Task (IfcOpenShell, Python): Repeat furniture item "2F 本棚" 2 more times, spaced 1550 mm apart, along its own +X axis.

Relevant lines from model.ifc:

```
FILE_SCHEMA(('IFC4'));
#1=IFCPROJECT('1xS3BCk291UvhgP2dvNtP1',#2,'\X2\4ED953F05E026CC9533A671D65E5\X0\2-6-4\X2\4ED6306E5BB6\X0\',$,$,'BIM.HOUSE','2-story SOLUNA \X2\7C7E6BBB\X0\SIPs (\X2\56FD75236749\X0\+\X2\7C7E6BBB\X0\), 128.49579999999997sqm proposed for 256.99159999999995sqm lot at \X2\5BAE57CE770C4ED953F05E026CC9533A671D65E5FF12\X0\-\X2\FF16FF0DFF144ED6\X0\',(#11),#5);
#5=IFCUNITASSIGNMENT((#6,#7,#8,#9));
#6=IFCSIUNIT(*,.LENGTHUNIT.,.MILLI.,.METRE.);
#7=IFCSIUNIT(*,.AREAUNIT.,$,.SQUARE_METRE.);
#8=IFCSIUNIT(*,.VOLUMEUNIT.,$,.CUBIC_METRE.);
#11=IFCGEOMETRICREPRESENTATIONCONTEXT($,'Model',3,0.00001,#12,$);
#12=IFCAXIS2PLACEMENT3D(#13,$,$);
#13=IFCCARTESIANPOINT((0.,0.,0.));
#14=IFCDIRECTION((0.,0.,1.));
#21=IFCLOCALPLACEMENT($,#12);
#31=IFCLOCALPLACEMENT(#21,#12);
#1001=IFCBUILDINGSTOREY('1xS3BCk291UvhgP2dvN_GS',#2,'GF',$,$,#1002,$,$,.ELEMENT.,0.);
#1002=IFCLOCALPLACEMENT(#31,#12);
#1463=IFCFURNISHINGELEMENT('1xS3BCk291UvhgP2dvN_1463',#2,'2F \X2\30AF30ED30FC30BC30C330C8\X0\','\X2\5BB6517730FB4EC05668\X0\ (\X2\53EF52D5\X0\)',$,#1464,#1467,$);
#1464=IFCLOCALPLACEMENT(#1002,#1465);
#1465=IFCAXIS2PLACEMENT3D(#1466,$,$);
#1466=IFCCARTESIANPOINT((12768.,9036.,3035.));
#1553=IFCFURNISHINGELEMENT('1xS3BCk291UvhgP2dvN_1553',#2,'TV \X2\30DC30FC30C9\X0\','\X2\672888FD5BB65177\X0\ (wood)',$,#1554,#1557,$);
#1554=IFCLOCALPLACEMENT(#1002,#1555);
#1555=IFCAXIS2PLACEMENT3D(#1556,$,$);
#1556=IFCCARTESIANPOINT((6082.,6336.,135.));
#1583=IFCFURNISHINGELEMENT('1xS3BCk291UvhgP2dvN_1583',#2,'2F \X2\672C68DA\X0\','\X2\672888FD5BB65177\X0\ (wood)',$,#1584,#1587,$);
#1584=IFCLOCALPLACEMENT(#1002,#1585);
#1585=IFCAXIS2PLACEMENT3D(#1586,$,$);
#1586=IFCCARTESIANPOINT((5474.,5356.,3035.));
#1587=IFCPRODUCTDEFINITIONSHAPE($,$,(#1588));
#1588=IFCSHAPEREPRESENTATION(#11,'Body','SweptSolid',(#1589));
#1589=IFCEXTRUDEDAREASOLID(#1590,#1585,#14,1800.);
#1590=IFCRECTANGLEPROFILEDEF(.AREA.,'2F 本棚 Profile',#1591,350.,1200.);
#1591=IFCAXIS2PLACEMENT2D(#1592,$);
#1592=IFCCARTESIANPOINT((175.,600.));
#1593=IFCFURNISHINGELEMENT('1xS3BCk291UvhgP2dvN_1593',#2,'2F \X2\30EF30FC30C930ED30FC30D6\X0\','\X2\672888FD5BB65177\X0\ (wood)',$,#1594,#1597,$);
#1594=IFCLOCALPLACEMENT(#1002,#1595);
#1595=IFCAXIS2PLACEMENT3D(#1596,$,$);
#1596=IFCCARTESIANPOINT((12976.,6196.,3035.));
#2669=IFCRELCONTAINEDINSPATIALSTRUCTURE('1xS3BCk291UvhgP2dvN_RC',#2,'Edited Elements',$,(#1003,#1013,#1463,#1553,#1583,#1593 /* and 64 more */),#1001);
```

```python
import ifcopenshell
import ifcopenshell.api.geometry
import ifcopenshell.api.root
import ifcopenshell.util.element
import ifcopenshell.util.placement
import ifcopenshell.util.unit

model = ifcopenshell.open("model.ifc")
unit_scale = ifcopenshell.util.unit.calculate_unit_scale(model)


def reuse_history(source, copy):
    """copy_class also copies each property set's owner history, people and application; keep the originals."""
    for rel in copy.IsDefinedBy:
        if rel.is_a("IfcRelDefinesByProperties") and (history := rel.RelatingPropertyDefinition.OwnerHistory):
            rel.RelatingPropertyDefinition.OwnerHistory = source.OwnerHistory
            ifcopenshell.util.element.remove_deep2(model, history)


source = model.by_id(1583)
base = ifcopenshell.util.placement.get_local_placement(source.ObjectPlacement)
step = base[:3, 0] * 1.55 / unit_scale

for i in range(1, 3):
    copy = ifcopenshell.api.root.copy_class(model, product=source)
    copy.Representation = ifcopenshell.util.element.copy_deep(
        model, source.Representation, exclude=["IfcGeometricRepresentationContext", "IfcRepresentationMap"]
    )
    reuse_history(source, copy)
    matrix = base.copy()
    matrix[:3, 3] += i * step
    print("added at", matrix[:3, 3].round(3) + 0.0)
    ifcopenshell.api.geometry.edit_object_placement(model, product=copy, matrix=matrix, is_si=False)

model.write("model_updated.ifc")
```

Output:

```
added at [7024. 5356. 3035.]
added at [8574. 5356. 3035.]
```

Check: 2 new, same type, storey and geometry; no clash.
